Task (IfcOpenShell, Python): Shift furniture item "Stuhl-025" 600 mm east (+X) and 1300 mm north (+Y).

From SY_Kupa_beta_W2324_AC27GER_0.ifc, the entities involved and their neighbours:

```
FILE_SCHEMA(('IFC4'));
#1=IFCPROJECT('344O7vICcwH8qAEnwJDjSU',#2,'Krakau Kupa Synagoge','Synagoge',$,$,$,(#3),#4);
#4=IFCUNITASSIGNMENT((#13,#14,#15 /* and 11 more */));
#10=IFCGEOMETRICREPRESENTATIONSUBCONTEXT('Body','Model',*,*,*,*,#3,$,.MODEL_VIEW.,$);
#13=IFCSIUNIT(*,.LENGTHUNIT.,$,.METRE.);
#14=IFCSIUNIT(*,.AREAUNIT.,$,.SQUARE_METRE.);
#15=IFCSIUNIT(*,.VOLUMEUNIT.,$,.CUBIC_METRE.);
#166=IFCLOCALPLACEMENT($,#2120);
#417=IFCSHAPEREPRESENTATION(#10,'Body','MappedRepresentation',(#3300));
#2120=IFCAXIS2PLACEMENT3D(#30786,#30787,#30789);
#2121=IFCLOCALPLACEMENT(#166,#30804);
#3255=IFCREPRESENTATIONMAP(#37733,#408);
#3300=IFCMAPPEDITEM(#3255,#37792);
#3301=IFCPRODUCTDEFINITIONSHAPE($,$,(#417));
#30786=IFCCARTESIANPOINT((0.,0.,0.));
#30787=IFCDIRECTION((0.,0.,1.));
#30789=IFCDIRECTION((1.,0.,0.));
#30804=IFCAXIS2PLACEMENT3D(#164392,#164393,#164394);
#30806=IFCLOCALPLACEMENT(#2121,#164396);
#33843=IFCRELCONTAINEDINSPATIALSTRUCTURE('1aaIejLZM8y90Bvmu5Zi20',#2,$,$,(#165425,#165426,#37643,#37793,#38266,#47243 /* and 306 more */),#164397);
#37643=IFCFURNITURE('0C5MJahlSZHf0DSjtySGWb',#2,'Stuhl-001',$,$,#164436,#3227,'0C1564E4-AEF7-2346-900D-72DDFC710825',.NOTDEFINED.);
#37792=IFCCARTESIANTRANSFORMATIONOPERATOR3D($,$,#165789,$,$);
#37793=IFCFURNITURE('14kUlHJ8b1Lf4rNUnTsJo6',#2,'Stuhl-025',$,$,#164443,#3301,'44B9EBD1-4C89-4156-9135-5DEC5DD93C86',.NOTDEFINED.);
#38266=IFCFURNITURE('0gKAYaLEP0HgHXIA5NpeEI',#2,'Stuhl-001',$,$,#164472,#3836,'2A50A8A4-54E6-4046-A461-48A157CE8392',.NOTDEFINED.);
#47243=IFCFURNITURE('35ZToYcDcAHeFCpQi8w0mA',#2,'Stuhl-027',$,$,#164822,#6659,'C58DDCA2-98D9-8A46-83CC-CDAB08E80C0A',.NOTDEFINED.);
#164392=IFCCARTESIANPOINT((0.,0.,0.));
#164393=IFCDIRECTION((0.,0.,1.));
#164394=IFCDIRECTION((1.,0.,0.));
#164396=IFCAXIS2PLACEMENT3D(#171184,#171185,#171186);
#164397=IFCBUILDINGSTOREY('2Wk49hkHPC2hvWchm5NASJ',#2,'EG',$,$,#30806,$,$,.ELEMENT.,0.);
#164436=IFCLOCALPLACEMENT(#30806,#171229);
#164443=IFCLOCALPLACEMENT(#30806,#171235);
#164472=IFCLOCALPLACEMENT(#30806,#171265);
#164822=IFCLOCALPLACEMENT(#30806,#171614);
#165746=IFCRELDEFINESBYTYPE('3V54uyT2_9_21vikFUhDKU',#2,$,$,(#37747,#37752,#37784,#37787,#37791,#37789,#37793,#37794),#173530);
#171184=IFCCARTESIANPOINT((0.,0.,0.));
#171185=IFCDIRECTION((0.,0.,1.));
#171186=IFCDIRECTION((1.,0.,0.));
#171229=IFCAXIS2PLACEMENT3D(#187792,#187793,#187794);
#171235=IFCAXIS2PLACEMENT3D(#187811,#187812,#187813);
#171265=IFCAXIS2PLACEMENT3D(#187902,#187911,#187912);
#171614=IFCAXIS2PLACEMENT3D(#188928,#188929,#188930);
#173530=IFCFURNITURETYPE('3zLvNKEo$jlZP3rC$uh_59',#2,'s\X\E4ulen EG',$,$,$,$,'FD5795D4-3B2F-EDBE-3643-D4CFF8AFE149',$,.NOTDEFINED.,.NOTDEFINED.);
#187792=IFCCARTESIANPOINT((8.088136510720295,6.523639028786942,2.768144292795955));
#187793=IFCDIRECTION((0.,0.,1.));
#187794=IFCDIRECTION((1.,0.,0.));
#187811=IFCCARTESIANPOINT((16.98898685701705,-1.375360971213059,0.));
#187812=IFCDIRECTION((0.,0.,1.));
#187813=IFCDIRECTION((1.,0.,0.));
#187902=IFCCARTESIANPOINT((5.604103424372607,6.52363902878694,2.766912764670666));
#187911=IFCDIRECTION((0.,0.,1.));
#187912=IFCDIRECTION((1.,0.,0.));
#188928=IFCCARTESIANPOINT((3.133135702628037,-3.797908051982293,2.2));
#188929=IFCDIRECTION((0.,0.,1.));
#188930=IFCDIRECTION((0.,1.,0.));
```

```python
import ifcopenshell
import ifcopenshell.api.geometry
import ifcopenshell.util.placement
import ifcopenshell.util.unit

model = ifcopenshell.open("SY_Kupa_beta_W2324_AC27GER_0.ifc")
unit_scale = ifcopenshell.util.unit.calculate_unit_scale(model)

item = model.by_id(37793)
matrix = ifcopenshell.util.placement.get_local_placement(item.ObjectPlacement)
matrix[0, 3] += 0.6 / unit_scale
matrix[1, 3] += 1.3 / unit_scale
ifcopenshell.api.geometry.edit_object_placement(model, product=item, matrix=matrix, is_si=False)

print(ifcopenshell.util.placement.get_local_placement(item.ObjectPlacement).round(3) + 0.0)

model.write("SY_Kupa_beta_W2324_AC27GER_0_v2.ifc")
```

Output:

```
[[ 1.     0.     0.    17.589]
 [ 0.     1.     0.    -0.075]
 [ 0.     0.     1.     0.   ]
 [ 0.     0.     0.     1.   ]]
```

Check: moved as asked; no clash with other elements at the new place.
